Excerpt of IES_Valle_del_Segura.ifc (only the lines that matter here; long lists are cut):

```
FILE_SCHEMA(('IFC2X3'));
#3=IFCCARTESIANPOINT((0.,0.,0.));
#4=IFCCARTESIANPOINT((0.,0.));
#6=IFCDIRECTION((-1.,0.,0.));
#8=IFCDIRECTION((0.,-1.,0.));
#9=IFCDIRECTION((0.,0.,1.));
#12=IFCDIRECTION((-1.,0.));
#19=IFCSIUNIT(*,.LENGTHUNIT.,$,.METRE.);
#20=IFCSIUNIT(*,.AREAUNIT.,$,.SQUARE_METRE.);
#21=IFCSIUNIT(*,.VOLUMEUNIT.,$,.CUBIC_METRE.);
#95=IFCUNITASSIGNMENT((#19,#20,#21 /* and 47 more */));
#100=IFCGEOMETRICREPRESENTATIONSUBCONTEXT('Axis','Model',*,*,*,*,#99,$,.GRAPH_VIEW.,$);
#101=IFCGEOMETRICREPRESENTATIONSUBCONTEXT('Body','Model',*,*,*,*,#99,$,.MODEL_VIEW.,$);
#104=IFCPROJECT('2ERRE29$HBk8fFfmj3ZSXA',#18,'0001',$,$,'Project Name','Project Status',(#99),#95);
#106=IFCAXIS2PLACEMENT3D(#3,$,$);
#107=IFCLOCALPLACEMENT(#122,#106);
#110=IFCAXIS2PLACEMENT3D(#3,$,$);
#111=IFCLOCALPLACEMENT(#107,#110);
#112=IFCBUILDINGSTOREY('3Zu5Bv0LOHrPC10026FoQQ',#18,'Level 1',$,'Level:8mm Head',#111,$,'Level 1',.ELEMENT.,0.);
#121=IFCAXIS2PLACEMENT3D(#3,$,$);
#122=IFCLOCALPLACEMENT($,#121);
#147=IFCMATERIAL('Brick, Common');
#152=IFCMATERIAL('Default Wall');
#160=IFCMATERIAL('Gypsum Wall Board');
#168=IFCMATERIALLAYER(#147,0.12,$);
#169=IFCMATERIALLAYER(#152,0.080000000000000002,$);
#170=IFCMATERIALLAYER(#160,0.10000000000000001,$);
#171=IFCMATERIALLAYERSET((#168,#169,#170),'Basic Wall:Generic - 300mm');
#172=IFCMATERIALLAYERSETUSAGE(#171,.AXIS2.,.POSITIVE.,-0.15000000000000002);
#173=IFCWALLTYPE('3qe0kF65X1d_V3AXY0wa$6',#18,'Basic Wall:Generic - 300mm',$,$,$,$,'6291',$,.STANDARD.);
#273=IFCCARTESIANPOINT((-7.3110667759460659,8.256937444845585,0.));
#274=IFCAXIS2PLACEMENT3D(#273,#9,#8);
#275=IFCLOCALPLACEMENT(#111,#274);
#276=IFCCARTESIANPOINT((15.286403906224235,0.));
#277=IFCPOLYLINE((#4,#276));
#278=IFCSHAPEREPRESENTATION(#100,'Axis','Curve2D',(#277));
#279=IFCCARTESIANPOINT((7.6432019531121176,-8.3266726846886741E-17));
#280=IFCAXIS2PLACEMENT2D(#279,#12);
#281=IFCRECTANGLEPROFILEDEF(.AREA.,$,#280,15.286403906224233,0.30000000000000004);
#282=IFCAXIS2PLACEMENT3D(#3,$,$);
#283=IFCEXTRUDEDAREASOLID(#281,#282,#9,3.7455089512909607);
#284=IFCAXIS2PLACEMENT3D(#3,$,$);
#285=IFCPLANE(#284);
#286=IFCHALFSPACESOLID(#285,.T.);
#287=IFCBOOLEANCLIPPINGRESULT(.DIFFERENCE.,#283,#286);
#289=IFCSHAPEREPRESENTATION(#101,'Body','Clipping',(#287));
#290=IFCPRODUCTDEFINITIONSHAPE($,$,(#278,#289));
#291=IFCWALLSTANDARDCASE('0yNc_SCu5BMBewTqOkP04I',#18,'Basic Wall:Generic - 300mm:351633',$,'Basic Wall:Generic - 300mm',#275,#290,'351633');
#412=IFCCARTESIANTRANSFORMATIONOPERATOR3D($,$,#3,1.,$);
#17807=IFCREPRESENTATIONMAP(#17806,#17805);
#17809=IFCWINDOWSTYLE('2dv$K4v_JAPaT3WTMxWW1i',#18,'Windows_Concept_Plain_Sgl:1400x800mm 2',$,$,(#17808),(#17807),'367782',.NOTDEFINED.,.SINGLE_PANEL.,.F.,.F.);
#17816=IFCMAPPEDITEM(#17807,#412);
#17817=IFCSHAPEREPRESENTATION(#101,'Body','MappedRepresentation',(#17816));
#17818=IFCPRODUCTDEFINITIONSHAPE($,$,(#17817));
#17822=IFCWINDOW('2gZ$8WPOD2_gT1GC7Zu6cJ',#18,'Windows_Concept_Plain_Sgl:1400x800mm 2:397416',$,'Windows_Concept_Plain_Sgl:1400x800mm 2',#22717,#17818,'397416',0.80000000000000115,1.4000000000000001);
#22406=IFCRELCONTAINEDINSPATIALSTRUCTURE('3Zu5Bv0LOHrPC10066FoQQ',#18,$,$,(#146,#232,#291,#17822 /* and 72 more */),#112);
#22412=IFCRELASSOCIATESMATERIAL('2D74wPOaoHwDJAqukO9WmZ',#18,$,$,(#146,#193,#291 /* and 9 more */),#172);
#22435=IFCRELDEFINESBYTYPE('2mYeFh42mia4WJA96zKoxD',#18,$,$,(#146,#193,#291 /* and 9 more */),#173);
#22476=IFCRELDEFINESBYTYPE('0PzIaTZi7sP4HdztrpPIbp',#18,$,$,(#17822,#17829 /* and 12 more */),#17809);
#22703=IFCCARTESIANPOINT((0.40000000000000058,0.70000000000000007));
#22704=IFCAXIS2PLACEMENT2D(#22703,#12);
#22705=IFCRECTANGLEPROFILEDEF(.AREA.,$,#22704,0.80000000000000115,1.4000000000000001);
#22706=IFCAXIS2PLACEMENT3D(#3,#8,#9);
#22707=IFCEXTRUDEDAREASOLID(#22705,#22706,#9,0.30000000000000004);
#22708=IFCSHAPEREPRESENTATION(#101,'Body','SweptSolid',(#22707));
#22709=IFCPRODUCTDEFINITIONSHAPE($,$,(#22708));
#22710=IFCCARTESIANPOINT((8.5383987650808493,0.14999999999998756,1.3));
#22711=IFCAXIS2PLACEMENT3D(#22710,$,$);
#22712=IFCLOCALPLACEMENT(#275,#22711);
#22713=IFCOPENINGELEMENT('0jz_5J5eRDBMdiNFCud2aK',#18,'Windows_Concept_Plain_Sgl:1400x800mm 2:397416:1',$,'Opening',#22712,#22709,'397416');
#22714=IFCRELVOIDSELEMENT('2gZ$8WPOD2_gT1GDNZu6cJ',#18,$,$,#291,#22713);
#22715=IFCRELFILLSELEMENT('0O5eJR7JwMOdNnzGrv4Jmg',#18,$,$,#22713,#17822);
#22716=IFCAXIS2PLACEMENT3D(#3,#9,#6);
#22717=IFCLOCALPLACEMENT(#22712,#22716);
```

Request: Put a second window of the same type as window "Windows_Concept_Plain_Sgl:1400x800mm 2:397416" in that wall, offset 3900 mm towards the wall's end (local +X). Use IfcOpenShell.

```python
import ifcopenshell
import ifcopenshell.api.feature
import ifcopenshell.api.geometry
import ifcopenshell.api.root
import ifcopenshell.geom
import ifcopenshell.util.element
import ifcopenshell.util.placement
import ifcopenshell.util.shape
import ifcopenshell.util.unit

model = ifcopenshell.open("IES_Valle_del_Segura.ifc")
unit_scale = ifcopenshell.util.unit.calculate_unit_scale(model)
settings = ifcopenshell.geom.settings()


def volume(element):
    """Net volume in cubic metres, openings subtracted."""
    shape = ifcopenshell.geom.create_shape(settings, element)
    return ifcopenshell.util.shape.get_volume(shape.geometry)


window = model.by_guid("2gZ$8WPOD2_gT1GC7Zu6cJ")
opening = window.FillsVoids[0].RelatingOpeningElement
wall = opening.VoidsElements[0].RelatingBuildingElement
before = volume(wall)
shift = ifcopenshell.util.placement.get_local_placement(wall.ObjectPlacement)[:3, 0] * 3.9 / unit_scale

# copy_class copies the void relationship, type, container and properties, but no geometry.
new_opening = ifcopenshell.api.root.copy_class(model, product=opening)
new_opening.Representation = ifcopenshell.util.element.copy_deep(
    model, opening.Representation, exclude=["IfcGeometricRepresentationContext", "IfcRepresentationMap"]
)
new_opening.Name = "Windows_Concept_Plain_Sgl:1400x800mm 2"
new_opening.Tag = None
new_window = ifcopenshell.api.root.copy_class(model, product=window)
new_window.Representation = ifcopenshell.util.element.copy_deep(
    model, window.Representation, exclude=["IfcGeometricRepresentationContext", "IfcRepresentationMap"]
)
new_window.Name = "Windows_Concept_Plain_Sgl:1400x800mm 2"
new_window.Tag = None
fills = ifcopenshell.api.feature.add_filling(model, opening=new_opening, element=new_window)
fills.OwnerHistory = new_window.OwnerHistory  # required in IFC2X3

for old, new in ((opening, new_opening), (window, new_window)):
    matrix = ifcopenshell.util.placement.get_local_placement(old.ObjectPlacement)
    matrix[:3, 3] += shift
    ifcopenshell.api.geometry.edit_object_placement(model, product=new, matrix=matrix, is_si=False)

after = volume(wall)

print(f"wall volume {before:.3f} -> {after:.3f} m3")

model.write("IES_Valle_del_Segura-out.ifc")
```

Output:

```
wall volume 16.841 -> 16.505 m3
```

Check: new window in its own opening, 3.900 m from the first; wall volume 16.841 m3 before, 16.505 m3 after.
